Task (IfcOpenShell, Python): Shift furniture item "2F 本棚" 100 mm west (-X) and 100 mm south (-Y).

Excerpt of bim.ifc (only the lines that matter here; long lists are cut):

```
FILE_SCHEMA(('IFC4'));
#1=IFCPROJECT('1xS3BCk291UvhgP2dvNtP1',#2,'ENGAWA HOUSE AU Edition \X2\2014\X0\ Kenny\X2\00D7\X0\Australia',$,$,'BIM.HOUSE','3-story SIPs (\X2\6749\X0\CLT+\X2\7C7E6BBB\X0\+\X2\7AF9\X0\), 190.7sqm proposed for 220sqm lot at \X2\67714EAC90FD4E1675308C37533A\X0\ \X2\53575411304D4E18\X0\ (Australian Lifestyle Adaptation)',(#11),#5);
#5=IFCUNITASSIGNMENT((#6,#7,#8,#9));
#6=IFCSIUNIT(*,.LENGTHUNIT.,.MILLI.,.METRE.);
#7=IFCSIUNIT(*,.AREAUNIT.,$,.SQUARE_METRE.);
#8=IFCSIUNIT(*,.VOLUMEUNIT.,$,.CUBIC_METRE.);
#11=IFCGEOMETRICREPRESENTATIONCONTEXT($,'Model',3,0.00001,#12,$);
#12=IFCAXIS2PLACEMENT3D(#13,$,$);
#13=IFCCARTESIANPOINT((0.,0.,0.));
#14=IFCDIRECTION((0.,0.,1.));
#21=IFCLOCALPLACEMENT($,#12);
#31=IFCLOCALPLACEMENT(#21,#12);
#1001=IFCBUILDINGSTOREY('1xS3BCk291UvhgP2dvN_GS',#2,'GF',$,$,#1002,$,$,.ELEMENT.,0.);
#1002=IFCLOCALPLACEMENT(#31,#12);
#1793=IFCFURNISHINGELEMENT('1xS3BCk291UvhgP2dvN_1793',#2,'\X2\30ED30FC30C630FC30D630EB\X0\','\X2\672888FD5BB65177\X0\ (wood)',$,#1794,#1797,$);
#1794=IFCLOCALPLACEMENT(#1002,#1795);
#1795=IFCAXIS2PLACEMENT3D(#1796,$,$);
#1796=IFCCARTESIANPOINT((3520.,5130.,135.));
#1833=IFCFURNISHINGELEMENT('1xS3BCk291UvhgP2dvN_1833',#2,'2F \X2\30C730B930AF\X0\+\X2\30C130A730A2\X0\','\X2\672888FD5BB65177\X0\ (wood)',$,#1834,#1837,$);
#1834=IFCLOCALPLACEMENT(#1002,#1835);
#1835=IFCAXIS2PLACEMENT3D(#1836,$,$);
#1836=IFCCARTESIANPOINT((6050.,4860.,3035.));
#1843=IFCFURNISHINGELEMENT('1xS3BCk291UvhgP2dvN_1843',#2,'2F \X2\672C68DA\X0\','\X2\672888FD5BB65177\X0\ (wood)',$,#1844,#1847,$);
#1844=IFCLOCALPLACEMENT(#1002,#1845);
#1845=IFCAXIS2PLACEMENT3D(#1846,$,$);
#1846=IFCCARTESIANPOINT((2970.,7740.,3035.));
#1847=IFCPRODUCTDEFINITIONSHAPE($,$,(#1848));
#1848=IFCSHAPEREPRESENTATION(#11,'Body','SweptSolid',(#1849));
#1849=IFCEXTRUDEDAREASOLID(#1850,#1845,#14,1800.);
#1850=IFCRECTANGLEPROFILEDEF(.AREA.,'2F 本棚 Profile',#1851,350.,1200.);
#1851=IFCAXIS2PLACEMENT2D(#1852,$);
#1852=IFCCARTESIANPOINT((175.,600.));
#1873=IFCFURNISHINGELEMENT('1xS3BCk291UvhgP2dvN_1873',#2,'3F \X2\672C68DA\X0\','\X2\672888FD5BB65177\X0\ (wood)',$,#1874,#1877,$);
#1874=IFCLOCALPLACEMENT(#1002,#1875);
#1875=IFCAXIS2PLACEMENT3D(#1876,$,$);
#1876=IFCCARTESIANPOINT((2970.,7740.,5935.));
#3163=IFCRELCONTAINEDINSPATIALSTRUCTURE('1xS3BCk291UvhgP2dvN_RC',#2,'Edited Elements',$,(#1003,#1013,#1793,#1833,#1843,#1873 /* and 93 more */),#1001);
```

```python
import ifcopenshell
import ifcopenshell.api.geometry
import ifcopenshell.util.placement
import ifcopenshell.util.unit

model = ifcopenshell.open("bim.ifc")
unit_scale = ifcopenshell.util.unit.calculate_unit_scale(model)

item = model.by_guid("1xS3BCk291UvhgP2dvN_1843")
matrix = ifcopenshell.util.placement.get_local_placement(item.ObjectPlacement)
matrix[0, 3] -= 0.1 / unit_scale
matrix[1, 3] -= 0.1 / unit_scale
ifcopenshell.api.geometry.edit_object_placement(model, product=item, matrix=matrix, is_si=False)

print(ifcopenshell.util.placement.get_local_placement(item.ObjectPlacement).round(3) + 0.0)

model.write("bim_edited.ifc")
```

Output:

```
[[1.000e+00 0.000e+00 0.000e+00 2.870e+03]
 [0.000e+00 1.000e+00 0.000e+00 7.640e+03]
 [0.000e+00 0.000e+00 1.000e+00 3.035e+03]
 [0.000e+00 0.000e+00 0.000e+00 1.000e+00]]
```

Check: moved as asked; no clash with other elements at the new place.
